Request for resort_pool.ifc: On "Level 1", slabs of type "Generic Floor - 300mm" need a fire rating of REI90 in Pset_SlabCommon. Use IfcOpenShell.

First a look at what the model holds.

```python
import ifcopenshell
import ifcopenshell.util.element

model = ifcopenshell.open("resort_pool.ifc")
print(model.schema)
storey = next(s for s in model.by_type("IfcBuildingStorey") if s.Name == "Level 1")
slabs = [e for e in ifcopenshell.util.element.get_decomposition(storey) if e.is_a("IfcSlab")]
seen = {}
for e in slabs:
    element_type = ifcopenshell.util.element.get_type(e)
    key = (element_type.Name if element_type != e and element_type else None, ifcopenshell.util.element.get_pset(e, "Pset_SlabCommon", "FireRating"))
    seen[key] = seen.get(key, 0) + 1
for (name, value), count in sorted(seen.items(), key=str):
    print(count, "x", name, "|", value)
```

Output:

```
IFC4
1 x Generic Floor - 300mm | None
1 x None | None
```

```python
import ifcopenshell
import ifcopenshell.api.pset
import ifcopenshell.util.element

model = ifcopenshell.open("resort_pool.ifc")

storey = next(s for s in model.by_type("IfcBuildingStorey") if s.Name == "Level 1")
slabs = [e for e in ifcopenshell.util.element.get_decomposition(storey) if e.is_a("IfcSlab")]

count = 0
for e in slabs:
    element_type = ifcopenshell.util.element.get_type(e)
    if element_type in (None, e) or element_type.Name != "Generic Floor - 300mm":
        continue
    # add_pset returns the element's existing set when there is one.
    pset = ifcopenshell.api.pset.add_pset(model, product=e, name="Pset_SlabCommon")
    ifcopenshell.api.pset.edit_pset(model, pset=pset, properties={"FireRating": "REI90"})
    count += 1

print(count, "slabs updated")

model.write("resort_pool_rev.ifc")
```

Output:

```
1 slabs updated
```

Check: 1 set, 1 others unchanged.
